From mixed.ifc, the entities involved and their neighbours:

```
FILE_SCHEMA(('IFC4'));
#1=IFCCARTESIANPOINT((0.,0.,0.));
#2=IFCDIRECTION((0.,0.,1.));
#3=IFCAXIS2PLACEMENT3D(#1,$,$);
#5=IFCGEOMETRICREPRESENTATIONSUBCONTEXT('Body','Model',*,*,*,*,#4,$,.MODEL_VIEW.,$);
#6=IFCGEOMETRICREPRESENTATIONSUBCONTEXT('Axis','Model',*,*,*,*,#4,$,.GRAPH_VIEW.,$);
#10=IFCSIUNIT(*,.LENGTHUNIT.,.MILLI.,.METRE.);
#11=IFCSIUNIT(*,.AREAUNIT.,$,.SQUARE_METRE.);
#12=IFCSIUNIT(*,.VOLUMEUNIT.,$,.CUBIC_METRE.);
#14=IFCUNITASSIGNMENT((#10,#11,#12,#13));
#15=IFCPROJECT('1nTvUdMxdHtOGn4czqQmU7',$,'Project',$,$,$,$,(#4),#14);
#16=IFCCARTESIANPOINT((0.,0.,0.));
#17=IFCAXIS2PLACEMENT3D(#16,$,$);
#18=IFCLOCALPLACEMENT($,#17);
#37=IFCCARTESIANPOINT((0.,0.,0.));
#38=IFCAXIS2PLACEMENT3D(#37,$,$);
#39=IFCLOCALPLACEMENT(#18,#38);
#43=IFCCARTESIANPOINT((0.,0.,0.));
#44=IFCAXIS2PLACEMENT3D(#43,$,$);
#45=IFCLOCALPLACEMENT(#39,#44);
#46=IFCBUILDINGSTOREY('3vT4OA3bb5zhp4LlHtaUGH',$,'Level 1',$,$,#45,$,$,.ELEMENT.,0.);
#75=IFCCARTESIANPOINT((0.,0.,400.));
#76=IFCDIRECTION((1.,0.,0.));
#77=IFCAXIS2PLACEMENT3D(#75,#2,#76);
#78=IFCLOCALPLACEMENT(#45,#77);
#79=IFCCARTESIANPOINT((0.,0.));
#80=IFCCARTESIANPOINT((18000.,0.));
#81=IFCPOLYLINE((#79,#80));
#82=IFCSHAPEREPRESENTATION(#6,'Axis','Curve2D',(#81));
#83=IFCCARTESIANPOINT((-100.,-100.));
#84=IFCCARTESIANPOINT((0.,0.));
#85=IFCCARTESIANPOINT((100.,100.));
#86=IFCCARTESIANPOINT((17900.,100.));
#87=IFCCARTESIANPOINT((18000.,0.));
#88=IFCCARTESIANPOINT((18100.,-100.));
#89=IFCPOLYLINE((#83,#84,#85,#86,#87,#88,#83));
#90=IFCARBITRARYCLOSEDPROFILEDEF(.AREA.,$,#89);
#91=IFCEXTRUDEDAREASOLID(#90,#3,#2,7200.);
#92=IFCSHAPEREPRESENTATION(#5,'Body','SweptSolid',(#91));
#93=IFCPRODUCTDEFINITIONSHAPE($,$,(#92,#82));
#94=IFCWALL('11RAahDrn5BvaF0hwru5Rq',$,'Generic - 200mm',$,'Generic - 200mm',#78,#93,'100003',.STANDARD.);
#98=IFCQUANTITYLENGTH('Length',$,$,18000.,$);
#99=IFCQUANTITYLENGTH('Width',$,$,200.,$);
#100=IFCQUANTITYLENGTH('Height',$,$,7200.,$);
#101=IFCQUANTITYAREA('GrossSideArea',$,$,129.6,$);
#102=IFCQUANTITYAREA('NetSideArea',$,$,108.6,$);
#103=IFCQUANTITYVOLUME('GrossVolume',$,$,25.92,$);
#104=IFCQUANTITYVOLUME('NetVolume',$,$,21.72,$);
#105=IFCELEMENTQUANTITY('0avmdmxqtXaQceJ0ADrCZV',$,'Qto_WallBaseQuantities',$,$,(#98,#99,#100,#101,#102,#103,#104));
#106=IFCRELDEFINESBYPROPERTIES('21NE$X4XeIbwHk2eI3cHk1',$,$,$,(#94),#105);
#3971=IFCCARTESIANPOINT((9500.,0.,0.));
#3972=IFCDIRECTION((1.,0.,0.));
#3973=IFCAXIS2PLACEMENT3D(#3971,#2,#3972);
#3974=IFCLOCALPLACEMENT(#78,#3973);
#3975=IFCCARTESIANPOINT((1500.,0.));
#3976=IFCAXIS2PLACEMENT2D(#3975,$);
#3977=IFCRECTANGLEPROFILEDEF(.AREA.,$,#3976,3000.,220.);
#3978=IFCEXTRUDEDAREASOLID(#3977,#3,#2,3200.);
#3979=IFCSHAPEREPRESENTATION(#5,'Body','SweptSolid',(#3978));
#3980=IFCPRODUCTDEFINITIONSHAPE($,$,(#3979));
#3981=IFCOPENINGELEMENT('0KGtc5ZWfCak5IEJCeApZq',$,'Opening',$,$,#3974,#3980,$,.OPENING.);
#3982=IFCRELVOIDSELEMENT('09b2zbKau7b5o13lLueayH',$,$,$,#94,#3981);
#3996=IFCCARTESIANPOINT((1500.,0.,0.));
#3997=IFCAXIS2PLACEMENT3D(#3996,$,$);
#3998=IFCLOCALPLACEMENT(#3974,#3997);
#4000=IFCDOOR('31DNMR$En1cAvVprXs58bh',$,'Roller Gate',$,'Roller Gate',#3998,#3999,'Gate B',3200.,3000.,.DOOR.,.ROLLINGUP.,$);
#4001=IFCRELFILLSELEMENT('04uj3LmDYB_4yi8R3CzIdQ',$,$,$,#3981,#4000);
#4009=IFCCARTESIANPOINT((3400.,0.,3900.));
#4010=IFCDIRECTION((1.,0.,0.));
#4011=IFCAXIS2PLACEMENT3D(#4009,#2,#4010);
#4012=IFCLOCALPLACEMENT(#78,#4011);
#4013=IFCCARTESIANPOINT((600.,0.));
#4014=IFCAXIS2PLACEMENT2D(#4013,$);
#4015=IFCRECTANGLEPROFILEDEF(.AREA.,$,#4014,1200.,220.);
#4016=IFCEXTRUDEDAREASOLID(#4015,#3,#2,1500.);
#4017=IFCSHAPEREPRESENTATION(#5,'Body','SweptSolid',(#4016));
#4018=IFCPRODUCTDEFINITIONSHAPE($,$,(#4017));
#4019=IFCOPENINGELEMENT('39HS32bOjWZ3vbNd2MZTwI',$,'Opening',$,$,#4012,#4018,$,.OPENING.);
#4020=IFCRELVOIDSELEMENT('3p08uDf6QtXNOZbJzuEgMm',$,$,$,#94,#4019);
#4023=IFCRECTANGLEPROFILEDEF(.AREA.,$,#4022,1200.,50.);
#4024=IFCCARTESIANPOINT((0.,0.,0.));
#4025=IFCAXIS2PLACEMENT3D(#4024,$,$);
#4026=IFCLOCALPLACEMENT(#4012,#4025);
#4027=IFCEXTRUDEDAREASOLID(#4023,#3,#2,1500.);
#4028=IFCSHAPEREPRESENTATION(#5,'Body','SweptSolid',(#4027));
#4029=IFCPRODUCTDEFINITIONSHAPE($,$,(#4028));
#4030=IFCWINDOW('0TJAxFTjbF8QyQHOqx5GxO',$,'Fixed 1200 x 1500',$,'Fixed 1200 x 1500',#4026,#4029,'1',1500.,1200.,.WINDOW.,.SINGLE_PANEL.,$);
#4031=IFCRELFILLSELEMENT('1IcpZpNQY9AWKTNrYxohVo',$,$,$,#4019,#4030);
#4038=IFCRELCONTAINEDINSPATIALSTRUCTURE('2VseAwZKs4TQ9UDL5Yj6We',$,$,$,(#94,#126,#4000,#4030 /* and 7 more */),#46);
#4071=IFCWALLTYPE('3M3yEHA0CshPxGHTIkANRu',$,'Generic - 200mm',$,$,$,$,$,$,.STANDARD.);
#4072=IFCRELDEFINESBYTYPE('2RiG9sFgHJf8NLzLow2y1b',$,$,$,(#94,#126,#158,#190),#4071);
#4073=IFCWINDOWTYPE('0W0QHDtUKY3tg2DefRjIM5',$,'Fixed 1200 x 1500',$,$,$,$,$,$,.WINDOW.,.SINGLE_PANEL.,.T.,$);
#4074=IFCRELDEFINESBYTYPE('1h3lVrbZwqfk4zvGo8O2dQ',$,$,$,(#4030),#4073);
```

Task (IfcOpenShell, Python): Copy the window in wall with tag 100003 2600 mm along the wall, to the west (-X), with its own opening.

```python
import ifcopenshell
import ifcopenshell.api.feature
import ifcopenshell.api.geometry
import ifcopenshell.api.pset
import ifcopenshell.api.root
import ifcopenshell.geom
import ifcopenshell.util.element
import ifcopenshell.util.placement
import ifcopenshell.util.shape
import ifcopenshell.util.unit

model = ifcopenshell.open("mixed.ifc")
area_scale = ifcopenshell.util.unit.calculate_unit_scale(model, "AREAUNIT")
volume_scale = ifcopenshell.util.unit.calculate_unit_scale(model, "VOLUMEUNIT")
settings = ifcopenshell.geom.settings()


def volume(element):
    """Net volume in cubic metres, openings subtracted."""
    shape = ifcopenshell.geom.create_shape(settings, element)
    return ifcopenshell.util.shape.get_volume(shape.geometry)


window = model.by_guid("0TJAxFTjbF8QyQHOqx5GxO")
opening = window.FillsVoids[0].RelatingOpeningElement
wall = opening.VoidsElements[0].RelatingBuildingElement
before = volume(wall)
shift = ifcopenshell.util.placement.get_local_placement(wall.ObjectPlacement)[:3, 0] * -2600.0

# copy_class copies the void relationship, type, container and properties, but no geometry.
new_opening = ifcopenshell.api.root.copy_class(model, product=opening)
new_opening.Representation = ifcopenshell.util.element.copy_deep(
    model, opening.Representation, exclude=["IfcGeometricRepresentationContext", "IfcRepresentationMap"]
)
new_window = ifcopenshell.api.root.copy_class(model, product=window)
new_window.Representation = ifcopenshell.util.element.copy_deep(
    model, window.Representation, exclude=["IfcGeometricRepresentationContext", "IfcRepresentationMap"]
)
new_window.Tag = None
ifcopenshell.api.feature.add_filling(model, opening=new_opening, element=new_window)

for old, new in ((opening, new_opening), (window, new_window)):
    matrix = ifcopenshell.util.placement.get_local_placement(old.ObjectPlacement)
    matrix[:3, 3] += shift
    ifcopenshell.api.geometry.edit_object_placement(model, product=new, matrix=matrix, is_si=False)

after = volume(wall)
thickness = 0.2  # wall thickness in metres

# Update the wall's stored quantities.
qto = model.by_id(ifcopenshell.util.element.get_pset(wall, "Qto_WallBaseQuantities", should_inherit=False)["id"])
ifcopenshell.api.pset.edit_qto(model, qto=qto, properties={
    "NetSideArea": after / thickness / area_scale,
    "NetVolume": after / volume_scale,
})

print(f"wall volume {before:.3f} -> {after:.3f} m3")

model.write("mixed_rev.ifc")
```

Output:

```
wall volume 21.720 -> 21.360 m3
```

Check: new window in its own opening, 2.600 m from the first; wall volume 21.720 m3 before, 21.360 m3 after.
